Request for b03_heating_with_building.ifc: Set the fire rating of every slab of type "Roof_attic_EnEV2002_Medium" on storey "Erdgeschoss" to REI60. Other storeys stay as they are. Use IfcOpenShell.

First a look at what the model holds.

```python
import ifcopenshell
import ifcopenshell.util.element

model = ifcopenshell.open("b03_heating_with_building.ifc")
print(model.schema)
storey = next(s for s in model.by_type("IfcBuildingStorey") if s.Name == "Erdgeschoss")
slabs = [e for e in ifcopenshell.util.element.get_decomposition(storey) if e.is_a("IfcSlab")]
seen = {}
for e in slabs:
    element_type = ifcopenshell.util.element.get_type(e)
    key = (element_type.Name if element_type != e and element_type else None, ifcopenshell.util.element.get_pset(e, "Pset_SlabCommon", "FireRating"))
    seen[key] = seen.get(key, 0) + 1
for (name, value), count in sorted(seen.items(), key=str):
    print(count, "x", name, "|", value)
```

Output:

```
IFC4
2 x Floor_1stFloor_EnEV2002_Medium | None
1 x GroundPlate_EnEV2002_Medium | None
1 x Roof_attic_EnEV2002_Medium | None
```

```python
import ifcopenshell
import ifcopenshell.api.pset
import ifcopenshell.util.element

model = ifcopenshell.open("b03_heating_with_building.ifc")

storey = next(s for s in model.by_type("IfcBuildingStorey") if s.Name == "Erdgeschoss")
slabs = [e for e in ifcopenshell.util.element.get_decomposition(storey) if e.is_a("IfcSlab")]

count = 0
for e in slabs:
    element_type = ifcopenshell.util.element.get_type(e)
    if element_type in (None, e) or element_type.Name != "Roof_attic_EnEV2002_Medium":
        continue
    # add_pset returns the element's existing set when there is one.
    pset = ifcopenshell.api.pset.add_pset(model, product=e, name="Pset_SlabCommon")
    ifcopenshell.api.pset.edit_pset(model, pset=pset, properties={"FireRating": "REI60"})
    count += 1

print(count, "slabs updated")

model.write("b03_heating_with_building-out.ifc")
```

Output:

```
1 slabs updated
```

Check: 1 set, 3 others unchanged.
